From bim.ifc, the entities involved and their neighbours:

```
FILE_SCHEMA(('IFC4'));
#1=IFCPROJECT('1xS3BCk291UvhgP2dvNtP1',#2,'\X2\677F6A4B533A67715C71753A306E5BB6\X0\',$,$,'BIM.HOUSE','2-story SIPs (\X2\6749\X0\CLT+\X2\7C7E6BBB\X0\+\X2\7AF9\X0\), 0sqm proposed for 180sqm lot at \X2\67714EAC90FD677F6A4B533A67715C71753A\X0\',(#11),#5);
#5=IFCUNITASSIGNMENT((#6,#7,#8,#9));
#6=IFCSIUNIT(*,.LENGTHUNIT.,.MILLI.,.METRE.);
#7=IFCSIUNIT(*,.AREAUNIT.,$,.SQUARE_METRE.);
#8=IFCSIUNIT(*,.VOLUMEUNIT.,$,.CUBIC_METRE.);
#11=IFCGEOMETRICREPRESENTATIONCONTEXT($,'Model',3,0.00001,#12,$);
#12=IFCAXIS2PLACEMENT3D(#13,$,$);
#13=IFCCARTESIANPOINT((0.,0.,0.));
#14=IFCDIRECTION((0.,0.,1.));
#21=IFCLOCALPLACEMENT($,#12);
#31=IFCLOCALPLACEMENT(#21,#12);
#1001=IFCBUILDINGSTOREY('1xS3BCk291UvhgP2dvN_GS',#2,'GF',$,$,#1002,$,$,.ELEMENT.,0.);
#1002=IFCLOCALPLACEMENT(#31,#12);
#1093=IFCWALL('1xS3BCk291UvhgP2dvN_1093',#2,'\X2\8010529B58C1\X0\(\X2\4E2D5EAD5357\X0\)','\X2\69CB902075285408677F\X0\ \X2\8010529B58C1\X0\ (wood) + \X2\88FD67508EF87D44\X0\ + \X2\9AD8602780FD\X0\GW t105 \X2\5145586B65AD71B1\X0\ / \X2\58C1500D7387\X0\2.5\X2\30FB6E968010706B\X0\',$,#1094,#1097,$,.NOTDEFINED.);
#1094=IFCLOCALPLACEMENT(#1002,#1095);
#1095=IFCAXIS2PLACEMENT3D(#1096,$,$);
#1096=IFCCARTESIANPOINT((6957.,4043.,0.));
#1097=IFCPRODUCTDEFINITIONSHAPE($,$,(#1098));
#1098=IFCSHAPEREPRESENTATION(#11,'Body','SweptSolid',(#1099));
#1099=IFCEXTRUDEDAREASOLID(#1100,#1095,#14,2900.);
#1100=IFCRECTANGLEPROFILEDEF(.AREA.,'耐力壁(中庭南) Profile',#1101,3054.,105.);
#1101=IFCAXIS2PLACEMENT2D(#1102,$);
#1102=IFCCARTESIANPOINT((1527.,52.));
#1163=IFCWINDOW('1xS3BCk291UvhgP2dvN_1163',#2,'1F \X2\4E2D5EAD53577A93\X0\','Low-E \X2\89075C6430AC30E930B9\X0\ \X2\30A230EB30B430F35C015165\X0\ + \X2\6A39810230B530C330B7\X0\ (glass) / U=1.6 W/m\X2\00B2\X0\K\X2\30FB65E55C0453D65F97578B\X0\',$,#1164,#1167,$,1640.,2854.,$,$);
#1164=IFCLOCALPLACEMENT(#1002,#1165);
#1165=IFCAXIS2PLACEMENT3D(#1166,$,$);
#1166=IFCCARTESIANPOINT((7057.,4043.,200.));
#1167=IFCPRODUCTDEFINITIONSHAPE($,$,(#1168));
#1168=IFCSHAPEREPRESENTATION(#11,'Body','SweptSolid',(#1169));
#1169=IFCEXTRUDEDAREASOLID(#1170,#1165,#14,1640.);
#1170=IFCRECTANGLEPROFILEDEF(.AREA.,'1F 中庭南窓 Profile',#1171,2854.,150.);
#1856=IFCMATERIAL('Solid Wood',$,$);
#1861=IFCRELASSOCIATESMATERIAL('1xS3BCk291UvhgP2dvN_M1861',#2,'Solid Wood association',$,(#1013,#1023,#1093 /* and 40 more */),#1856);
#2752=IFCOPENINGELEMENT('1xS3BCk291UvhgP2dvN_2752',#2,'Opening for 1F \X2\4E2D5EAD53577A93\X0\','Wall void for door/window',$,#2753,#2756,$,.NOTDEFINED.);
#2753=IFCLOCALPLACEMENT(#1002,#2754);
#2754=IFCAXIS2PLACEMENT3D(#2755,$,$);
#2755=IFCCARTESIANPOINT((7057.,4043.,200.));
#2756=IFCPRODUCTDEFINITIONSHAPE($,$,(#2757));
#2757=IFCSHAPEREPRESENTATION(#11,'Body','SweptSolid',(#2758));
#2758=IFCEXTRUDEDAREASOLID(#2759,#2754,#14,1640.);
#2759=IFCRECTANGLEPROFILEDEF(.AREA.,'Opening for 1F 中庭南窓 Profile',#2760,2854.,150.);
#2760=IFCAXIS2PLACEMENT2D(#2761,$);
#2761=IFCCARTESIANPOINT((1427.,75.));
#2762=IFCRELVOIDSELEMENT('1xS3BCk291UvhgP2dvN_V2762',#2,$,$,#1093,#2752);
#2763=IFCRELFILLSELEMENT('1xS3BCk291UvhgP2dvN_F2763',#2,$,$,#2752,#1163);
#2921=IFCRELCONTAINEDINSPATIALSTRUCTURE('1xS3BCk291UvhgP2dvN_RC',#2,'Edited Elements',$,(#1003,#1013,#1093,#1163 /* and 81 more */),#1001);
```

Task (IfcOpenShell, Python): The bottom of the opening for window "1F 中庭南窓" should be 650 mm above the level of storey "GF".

```python
import numpy as np
import ifcopenshell
import ifcopenshell.api.geometry
import ifcopenshell.geom
import ifcopenshell.util.element
import ifcopenshell.util.placement
import ifcopenshell.util.shape
import ifcopenshell.util.unit

model = ifcopenshell.open("bim.ifc")
unit_scale = ifcopenshell.util.unit.calculate_unit_scale(model)

window = model.by_guid("1xS3BCk291UvhgP2dvN_1163")
opening = window.FillsVoids[0].RelatingOpeningElement
storey = ifcopenshell.util.element.get_container(window, ifc_class="IfcBuildingStorey")
level = ifcopenshell.util.placement.get_local_placement(storey.ObjectPlacement)[2, 3]

# The opening's origin need not be at the sill, so measure its lowest point.
shape = ifcopenshell.geom.create_shape(ifcopenshell.geom.settings(), opening)
bottom = ifcopenshell.util.shape.get_shape_bottom_elevation(shape, shape.geometry) / unit_scale
dz = level + 650.0 - bottom

shift = np.array([0.0, 0.0, dz])
# The window is not placed relative to its opening, so move both.
for product in (opening, window):
    matrix = ifcopenshell.util.placement.get_local_placement(product.ObjectPlacement)
    matrix[:3, 3] += shift
    ifcopenshell.api.geometry.edit_object_placement(model, product=product, matrix=matrix, is_si=False)

print(f"moved by {dz * unit_scale:+.3f} m")

model.write("bim_v2.ifc")
```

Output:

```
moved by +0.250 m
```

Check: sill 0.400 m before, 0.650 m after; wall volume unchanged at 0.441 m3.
